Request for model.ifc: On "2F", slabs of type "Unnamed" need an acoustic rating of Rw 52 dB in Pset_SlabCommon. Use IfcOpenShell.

First a look at what the model holds.

```python
import ifcopenshell
import ifcopenshell.util.element

model = ifcopenshell.open("model.ifc")
print(model.schema)
storey = next(s for s in model.by_type("IfcBuildingStorey") if s.Name == "2F")
slabs = [e for e in ifcopenshell.util.element.get_decomposition(storey) if e.is_a("IfcSlab")]
seen = {}
for e in slabs:
    element_type = ifcopenshell.util.element.get_type(e)
    key = (element_type.Name if element_type != e and element_type else None, ifcopenshell.util.element.get_pset(e, "Pset_SlabCommon", "AcousticRating"))
    seen[key] = seen.get(key, 0) + 1
for (name, value), count in sorted(seen.items(), key=str):
    print(count, "x", name, "|", value)
```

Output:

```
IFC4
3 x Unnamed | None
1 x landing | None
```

```python
import ifcopenshell
import ifcopenshell.api.pset
import ifcopenshell.util.element

model = ifcopenshell.open("model.ifc")

storey = next(s for s in model.by_type("IfcBuildingStorey") if s.Name == "2F")
slabs = [e for e in ifcopenshell.util.element.get_decomposition(storey) if e.is_a("IfcSlab")]

count = 0
for e in slabs:
    element_type = ifcopenshell.util.element.get_type(e)
    if element_type in (None, e) or element_type.Name != "Unnamed":
        continue
    # add_pset returns the element's existing set when there is one.
    pset = ifcopenshell.api.pset.add_pset(model, product=e, name="Pset_SlabCommon")
    ifcopenshell.api.pset.edit_pset(model, pset=pset, properties={"AcousticRating": "Rw 52 dB"})
    count += 1

print(count, "slabs updated")

model.write("model_edited.ifc")
```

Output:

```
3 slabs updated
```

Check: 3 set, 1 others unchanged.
